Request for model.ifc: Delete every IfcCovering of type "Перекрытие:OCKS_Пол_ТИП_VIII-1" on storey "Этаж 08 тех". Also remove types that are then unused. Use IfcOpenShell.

First a look at what the model holds.

```python
import ifcopenshell
import ifcopenshell.util.element

model = ifcopenshell.open("model.ifc")
print(model.schema)
storey = next(s for s in model.by_type("IfcBuildingStorey") if s.Name == "Этаж 08 тех")
coverings = [e for e in ifcopenshell.util.element.get_decomposition(storey) if e.is_a("IfcCovering")]
seen = {}
for e in coverings:
    element_type = ifcopenshell.util.element.get_type(e)
    name = element_type.Name if element_type not in (None, e) else None
    seen[name] = seen.get(name, 0) + 1
for name, count in sorted(seen.items(), key=str):
    print(count, "x", name)
```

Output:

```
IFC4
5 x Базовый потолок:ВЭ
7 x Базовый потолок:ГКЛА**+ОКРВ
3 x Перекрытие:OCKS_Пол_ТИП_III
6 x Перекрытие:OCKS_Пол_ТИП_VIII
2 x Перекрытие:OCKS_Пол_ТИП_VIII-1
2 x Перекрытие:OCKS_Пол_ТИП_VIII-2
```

```python
import ifcopenshell
import ifcopenshell.api.root
import ifcopenshell.util.element

model = ifcopenshell.open("model.ifc")

storey = next(s for s in model.by_type("IfcBuildingStorey") if s.Name == "Этаж 08 тех")
coverings = [e for e in ifcopenshell.util.element.get_decomposition(storey) if e.is_a("IfcCovering")]
targets = [e for e in coverings if (t := ifcopenshell.util.element.get_type(e)) not in (None, e) and t.Name == "Перекрытие:OCKS_Пол_ТИП_VIII-1"]
types = {ifcopenshell.util.element.get_type(e) for e in targets} - {None, *targets}

for e in targets:
    ifcopenshell.api.root.remove_product(model, product=e)
print(len(targets), "removed")

unused = [t for t in types if not ifcopenshell.util.element.get_types(t)]
for t in unused:
    ifcopenshell.api.root.remove_product(model, product=t)
print(len(unused), "unused types removed")

model.write("model_edited.ifc")
```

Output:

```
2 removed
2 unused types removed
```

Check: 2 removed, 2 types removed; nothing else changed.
